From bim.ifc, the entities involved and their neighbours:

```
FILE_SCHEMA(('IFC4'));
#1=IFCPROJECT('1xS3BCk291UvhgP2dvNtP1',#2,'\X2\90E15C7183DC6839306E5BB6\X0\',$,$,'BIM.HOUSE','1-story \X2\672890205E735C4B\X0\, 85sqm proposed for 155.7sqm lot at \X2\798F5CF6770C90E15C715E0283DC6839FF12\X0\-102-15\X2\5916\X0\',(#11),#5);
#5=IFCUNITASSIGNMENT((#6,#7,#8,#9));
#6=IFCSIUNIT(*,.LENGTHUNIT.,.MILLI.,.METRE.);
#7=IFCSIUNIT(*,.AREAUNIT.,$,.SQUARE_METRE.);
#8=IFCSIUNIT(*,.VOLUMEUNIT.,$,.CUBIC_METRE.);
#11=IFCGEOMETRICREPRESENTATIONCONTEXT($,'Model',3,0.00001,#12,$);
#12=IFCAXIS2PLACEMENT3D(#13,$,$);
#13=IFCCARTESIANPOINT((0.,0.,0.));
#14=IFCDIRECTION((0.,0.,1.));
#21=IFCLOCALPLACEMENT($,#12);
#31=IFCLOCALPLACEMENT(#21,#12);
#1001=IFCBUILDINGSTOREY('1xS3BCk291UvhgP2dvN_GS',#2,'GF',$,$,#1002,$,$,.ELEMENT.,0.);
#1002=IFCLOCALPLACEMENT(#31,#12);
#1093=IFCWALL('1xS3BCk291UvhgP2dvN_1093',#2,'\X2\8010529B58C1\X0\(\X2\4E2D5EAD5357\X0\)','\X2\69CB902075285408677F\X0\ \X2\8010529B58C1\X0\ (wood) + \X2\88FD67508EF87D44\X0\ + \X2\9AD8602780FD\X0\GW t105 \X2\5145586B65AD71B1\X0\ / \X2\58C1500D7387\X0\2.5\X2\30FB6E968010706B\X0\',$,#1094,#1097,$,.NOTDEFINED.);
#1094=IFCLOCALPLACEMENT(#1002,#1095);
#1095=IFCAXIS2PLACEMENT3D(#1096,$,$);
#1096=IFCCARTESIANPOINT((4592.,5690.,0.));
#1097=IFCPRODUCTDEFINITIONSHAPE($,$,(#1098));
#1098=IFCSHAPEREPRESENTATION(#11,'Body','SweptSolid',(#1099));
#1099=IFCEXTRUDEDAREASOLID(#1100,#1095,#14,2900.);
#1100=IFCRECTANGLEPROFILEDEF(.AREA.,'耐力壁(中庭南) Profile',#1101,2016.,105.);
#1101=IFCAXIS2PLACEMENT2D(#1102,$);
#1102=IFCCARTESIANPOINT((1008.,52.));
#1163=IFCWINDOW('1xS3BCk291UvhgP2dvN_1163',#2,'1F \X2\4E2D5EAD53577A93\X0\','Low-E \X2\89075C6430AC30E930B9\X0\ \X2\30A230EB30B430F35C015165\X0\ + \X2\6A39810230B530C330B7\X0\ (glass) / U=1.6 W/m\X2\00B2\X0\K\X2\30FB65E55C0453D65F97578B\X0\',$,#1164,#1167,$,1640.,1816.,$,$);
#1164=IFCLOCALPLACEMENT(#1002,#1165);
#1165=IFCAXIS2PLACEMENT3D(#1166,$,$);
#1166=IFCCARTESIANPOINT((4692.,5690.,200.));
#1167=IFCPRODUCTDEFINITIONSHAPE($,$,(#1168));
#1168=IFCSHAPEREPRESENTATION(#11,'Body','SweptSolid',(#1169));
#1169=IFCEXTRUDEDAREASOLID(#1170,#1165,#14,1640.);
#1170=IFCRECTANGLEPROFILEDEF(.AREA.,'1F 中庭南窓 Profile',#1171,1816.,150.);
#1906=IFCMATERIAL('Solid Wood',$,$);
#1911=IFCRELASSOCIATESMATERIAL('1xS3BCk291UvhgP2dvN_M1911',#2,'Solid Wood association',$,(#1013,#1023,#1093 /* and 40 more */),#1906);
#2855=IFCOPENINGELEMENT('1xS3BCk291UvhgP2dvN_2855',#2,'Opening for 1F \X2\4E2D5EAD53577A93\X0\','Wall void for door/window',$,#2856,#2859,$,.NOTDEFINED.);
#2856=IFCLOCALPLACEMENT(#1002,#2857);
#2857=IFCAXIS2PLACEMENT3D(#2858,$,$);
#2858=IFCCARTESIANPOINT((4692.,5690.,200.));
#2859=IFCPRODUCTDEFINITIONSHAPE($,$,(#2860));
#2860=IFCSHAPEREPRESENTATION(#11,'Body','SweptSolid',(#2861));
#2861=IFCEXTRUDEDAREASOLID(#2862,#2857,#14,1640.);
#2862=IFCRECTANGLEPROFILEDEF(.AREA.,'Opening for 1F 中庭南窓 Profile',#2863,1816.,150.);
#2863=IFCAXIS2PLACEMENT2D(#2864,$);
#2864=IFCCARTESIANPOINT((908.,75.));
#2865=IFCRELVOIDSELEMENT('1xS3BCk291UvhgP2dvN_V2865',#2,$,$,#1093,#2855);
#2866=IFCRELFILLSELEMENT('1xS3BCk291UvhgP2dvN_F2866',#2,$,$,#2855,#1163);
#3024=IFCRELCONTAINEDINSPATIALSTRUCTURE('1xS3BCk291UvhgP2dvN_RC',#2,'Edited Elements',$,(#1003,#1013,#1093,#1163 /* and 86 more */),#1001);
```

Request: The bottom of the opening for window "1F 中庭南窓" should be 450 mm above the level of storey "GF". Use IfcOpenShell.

```python
import numpy as np
import ifcopenshell
import ifcopenshell.api.geometry
import ifcopenshell.geom
import ifcopenshell.util.element
import ifcopenshell.util.placement
import ifcopenshell.util.shape
import ifcopenshell.util.unit

model = ifcopenshell.open("bim.ifc")
unit_scale = ifcopenshell.util.unit.calculate_unit_scale(model)

window = model.by_guid("1xS3BCk291UvhgP2dvN_1163")
opening = window.FillsVoids[0].RelatingOpeningElement
storey = ifcopenshell.util.element.get_container(window, ifc_class="IfcBuildingStorey")
level = ifcopenshell.util.placement.get_local_placement(storey.ObjectPlacement)[2, 3]

# The opening's origin need not be at the sill, so measure its lowest point.
shape = ifcopenshell.geom.create_shape(ifcopenshell.geom.settings(), opening)
bottom = ifcopenshell.util.shape.get_shape_bottom_elevation(shape, shape.geometry) / unit_scale
dz = level + 0.45 / unit_scale - bottom

shift = np.array([0.0, 0.0, dz])
# The window is not placed relative to its opening, so move both.
for product in (opening, window):
    matrix = ifcopenshell.util.placement.get_local_placement(product.ObjectPlacement)
    matrix[:3, 3] += shift
    ifcopenshell.api.geometry.edit_object_placement(model, product=product, matrix=matrix, is_si=False)

print(f"moved by {dz * unit_scale:+.3f} m")

model.write("bim_updated.ifc")
```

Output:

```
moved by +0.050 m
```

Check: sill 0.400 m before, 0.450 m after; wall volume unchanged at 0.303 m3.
